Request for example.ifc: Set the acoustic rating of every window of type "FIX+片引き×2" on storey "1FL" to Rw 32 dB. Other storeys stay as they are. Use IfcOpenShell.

First a look at what the model holds.

```python
import ifcopenshell
import ifcopenshell.util.element

model = ifcopenshell.open("example.ifc")
print(model.schema)
storey = next(s for s in model.by_type("IfcBuildingStorey") if s.Name == "1FL")
windows = [e for e in ifcopenshell.util.element.get_decomposition(storey) if e.is_a("IfcWindow")]
seen = {}
for e in windows:
    element_type = ifcopenshell.util.element.get_type(e)
    key = (element_type.Name if element_type != e and element_type else None, ifcopenshell.util.element.get_pset(e, "Pset_WindowCommon", "AcousticRating"))
    seen[key] = seen.get(key, 0) + 1
for (name, value), count in sorted(seen.items(), key=str):
    print(count, "x", name, "|", value)
```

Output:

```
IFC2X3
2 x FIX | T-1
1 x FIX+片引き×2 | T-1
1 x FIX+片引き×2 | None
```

```python
import ifcopenshell
import ifcopenshell.api.pset
import ifcopenshell.util.element

model = ifcopenshell.open("example.ifc")

storey = next(s for s in model.by_type("IfcBuildingStorey") if s.Name == "1FL")
windows = [e for e in ifcopenshell.util.element.get_decomposition(storey) if e.is_a("IfcWindow")]

count = 0
for e in windows:
    element_type = ifcopenshell.util.element.get_type(e)
    if element_type in (None, e) or element_type.Name != "FIX+片引き×2":
        continue
    # add_pset returns the element's existing set when there is one.
    pset = ifcopenshell.api.pset.add_pset(model, product=e, name="Pset_WindowCommon")
    ifcopenshell.api.pset.edit_pset(model, pset=pset, properties={"AcousticRating": "Rw 32 dB"})
    count += 1

print(count, "windows updated")

model.write("example_rev.ifc")
```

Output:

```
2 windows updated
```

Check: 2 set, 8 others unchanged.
